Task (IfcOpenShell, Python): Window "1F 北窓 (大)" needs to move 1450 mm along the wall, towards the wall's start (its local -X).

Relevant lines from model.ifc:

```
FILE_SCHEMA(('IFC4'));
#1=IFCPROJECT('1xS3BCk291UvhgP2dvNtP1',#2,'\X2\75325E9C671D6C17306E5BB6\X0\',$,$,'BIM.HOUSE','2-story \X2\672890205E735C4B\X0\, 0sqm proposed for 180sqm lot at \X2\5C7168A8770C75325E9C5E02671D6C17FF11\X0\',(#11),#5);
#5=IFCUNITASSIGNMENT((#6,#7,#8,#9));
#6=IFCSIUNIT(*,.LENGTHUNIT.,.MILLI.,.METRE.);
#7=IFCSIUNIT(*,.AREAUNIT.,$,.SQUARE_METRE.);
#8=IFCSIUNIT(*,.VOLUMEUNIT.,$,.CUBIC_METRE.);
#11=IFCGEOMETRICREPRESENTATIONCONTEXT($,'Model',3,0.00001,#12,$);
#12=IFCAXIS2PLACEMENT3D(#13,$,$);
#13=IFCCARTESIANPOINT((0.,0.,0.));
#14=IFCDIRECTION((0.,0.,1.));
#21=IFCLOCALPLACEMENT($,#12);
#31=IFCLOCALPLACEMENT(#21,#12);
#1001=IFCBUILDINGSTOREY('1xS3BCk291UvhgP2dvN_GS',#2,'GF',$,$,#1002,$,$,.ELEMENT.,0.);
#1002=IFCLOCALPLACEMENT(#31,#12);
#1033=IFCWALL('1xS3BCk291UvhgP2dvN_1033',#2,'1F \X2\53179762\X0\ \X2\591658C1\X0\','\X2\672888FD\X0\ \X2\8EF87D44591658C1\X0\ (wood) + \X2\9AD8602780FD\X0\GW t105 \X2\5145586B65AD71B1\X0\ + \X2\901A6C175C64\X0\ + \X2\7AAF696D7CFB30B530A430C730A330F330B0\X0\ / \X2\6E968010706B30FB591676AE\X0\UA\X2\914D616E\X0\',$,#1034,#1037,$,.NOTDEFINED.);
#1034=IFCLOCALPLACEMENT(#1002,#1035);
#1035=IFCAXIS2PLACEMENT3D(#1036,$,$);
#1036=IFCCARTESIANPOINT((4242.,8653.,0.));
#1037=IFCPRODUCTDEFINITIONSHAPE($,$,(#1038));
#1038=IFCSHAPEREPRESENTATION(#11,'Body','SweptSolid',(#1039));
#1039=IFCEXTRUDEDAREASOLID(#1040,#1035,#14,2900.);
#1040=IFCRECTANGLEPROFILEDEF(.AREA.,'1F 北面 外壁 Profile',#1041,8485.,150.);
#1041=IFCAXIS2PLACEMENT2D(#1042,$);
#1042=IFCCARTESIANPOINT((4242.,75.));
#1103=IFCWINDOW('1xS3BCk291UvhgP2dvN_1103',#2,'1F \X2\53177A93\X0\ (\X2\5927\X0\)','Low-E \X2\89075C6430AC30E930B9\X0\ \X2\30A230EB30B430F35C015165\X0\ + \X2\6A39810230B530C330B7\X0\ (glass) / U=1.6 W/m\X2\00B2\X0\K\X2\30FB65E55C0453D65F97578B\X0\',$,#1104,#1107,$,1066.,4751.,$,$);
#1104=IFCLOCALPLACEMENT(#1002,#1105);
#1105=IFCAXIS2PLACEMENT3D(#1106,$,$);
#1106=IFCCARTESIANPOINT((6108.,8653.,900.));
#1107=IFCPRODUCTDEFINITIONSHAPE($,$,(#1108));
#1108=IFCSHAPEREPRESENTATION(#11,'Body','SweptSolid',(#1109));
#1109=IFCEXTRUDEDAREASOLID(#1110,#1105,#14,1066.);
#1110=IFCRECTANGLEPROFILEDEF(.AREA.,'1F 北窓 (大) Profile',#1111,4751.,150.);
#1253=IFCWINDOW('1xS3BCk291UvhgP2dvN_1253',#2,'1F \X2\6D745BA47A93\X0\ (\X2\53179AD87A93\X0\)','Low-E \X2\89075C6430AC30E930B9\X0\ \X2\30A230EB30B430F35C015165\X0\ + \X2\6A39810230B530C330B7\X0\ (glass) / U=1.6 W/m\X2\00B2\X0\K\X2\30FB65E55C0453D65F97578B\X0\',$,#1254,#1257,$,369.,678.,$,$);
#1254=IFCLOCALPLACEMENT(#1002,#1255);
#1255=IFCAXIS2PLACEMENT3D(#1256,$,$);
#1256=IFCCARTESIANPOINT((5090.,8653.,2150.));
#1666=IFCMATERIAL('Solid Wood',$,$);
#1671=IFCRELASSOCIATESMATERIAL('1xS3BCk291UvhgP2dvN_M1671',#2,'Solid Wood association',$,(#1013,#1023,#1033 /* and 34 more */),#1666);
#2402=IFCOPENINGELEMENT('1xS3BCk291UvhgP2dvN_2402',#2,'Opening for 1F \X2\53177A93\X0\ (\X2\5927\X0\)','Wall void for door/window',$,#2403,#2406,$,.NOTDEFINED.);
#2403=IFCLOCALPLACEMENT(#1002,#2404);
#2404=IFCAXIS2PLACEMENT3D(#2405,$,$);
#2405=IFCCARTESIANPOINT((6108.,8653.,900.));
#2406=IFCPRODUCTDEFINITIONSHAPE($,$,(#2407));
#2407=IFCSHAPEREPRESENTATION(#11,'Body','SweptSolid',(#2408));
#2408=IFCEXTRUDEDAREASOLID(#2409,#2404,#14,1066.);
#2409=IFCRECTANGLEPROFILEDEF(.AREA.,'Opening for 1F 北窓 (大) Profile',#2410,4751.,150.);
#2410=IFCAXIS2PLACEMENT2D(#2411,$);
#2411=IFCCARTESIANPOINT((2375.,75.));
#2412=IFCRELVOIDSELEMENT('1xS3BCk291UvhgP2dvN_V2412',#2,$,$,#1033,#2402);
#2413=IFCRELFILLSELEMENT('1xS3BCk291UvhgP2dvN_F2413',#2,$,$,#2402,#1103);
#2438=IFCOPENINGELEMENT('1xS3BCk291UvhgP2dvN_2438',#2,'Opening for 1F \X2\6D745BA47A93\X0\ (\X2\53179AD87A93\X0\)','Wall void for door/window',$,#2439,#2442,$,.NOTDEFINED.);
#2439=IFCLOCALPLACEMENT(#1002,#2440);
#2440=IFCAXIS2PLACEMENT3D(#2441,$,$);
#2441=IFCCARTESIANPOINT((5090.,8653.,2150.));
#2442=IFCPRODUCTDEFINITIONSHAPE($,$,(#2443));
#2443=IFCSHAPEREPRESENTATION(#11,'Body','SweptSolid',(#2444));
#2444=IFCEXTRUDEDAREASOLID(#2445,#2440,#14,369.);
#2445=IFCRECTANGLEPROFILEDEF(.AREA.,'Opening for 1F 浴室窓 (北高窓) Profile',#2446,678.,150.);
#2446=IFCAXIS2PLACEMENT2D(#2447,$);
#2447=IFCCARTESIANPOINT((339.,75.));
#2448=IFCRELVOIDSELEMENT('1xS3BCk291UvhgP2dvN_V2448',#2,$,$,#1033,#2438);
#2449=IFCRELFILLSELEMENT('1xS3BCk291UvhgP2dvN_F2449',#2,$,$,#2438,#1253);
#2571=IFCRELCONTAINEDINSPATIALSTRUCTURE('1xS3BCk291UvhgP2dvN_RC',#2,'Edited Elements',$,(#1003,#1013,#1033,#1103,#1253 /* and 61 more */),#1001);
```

```python
import ifcopenshell
import ifcopenshell.api.geometry
import ifcopenshell.util.placement
import ifcopenshell.util.unit

model = ifcopenshell.open("model.ifc")
unit_scale = ifcopenshell.util.unit.calculate_unit_scale(model)

window = model.by_guid("1xS3BCk291UvhgP2dvN_1103")
opening = window.FillsVoids[0].RelatingOpeningElement
wall = opening.VoidsElements[0].RelatingBuildingElement

wall_matrix = ifcopenshell.util.placement.get_local_placement(wall.ObjectPlacement)
shift = wall_matrix[:3, 0] * -1.45 / unit_scale
before = ifcopenshell.util.placement.get_local_placement(window.ObjectPlacement)[:3, 3].copy()

# The window is not placed relative to its opening, so move both.
for product in (opening, window):
    matrix = ifcopenshell.util.placement.get_local_placement(product.ObjectPlacement)
    matrix[:3, 3] += shift
    ifcopenshell.api.geometry.edit_object_placement(model, product=product, matrix=matrix, is_si=False)

after = ifcopenshell.util.placement.get_local_placement(window.ObjectPlacement)[:3, 3]
print("window moved by", (after - before).round(3) + 0.0)

model.write("model_v2.ifc")
```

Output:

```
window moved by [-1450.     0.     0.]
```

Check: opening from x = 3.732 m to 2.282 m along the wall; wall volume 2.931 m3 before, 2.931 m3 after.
